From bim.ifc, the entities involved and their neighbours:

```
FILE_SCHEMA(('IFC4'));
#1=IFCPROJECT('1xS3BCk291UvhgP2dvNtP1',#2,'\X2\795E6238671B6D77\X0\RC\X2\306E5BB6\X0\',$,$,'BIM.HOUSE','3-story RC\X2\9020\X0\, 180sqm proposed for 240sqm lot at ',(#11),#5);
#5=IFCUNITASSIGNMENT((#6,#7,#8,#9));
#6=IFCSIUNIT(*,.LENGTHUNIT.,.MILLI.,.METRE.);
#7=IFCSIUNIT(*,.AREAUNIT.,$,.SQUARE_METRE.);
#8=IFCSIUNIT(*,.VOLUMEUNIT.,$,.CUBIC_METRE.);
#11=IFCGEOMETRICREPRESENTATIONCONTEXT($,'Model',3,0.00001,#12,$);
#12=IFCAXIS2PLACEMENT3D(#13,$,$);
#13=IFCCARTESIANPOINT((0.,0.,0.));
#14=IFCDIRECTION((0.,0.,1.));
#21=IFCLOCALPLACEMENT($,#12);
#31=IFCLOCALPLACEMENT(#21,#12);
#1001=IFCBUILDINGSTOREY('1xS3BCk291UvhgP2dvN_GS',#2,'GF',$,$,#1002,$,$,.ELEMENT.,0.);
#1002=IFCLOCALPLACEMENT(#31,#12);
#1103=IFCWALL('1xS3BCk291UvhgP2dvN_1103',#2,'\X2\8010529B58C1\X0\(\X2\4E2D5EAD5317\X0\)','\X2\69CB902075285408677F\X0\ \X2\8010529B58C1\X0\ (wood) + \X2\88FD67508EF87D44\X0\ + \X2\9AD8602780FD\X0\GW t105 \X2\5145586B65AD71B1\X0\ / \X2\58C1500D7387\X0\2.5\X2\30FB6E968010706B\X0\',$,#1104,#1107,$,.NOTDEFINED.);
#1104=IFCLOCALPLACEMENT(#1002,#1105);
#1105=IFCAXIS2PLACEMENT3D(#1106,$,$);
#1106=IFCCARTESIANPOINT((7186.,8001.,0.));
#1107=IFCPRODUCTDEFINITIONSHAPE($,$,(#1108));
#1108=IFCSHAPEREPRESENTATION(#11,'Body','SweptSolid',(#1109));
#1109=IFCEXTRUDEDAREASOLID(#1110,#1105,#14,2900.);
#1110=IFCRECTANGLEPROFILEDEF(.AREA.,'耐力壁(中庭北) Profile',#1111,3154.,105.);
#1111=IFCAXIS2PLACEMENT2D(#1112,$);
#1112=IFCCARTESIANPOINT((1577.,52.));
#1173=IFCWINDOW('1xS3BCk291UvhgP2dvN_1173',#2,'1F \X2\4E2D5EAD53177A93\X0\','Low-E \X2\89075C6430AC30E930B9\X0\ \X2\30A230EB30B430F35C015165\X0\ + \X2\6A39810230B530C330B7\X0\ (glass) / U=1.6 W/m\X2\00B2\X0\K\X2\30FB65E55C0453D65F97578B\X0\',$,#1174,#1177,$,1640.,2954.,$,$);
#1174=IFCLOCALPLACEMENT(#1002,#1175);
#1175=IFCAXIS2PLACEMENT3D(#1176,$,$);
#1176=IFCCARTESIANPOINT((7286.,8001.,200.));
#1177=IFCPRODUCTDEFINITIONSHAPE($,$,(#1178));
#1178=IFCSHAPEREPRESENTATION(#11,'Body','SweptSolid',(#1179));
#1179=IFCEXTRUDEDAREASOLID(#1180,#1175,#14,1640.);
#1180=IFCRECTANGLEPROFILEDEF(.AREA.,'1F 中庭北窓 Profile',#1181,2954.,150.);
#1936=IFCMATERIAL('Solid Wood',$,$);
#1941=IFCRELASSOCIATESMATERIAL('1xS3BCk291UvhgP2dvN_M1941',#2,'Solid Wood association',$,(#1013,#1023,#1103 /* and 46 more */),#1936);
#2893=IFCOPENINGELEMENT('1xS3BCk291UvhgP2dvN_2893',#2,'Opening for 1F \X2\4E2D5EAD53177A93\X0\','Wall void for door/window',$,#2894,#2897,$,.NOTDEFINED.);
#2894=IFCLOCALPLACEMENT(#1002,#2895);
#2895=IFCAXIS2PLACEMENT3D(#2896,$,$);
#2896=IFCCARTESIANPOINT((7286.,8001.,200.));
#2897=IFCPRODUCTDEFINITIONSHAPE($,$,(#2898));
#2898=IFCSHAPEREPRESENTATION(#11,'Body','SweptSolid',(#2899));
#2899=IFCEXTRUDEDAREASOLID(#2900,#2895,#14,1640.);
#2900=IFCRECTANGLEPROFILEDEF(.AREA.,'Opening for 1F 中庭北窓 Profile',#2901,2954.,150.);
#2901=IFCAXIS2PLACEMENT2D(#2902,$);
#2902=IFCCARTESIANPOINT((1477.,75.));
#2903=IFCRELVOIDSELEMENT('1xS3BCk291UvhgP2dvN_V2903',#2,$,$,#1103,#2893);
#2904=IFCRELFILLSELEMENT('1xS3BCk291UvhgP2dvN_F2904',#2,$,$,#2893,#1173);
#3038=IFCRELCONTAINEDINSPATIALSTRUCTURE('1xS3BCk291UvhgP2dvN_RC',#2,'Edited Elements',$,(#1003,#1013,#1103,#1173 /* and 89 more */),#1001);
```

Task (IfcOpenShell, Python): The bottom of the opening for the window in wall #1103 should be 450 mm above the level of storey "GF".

```python
import numpy as np
import ifcopenshell
import ifcopenshell.api.geometry
import ifcopenshell.geom
import ifcopenshell.util.element
import ifcopenshell.util.placement
import ifcopenshell.util.shape
import ifcopenshell.util.unit

model = ifcopenshell.open("bim.ifc")
unit_scale = ifcopenshell.util.unit.calculate_unit_scale(model)

window = model.by_guid("1xS3BCk291UvhgP2dvN_1173")
opening = window.FillsVoids[0].RelatingOpeningElement
storey = ifcopenshell.util.element.get_container(window, ifc_class="IfcBuildingStorey")
level = ifcopenshell.util.placement.get_local_placement(storey.ObjectPlacement)[2, 3]

# The opening's origin need not be at the sill, so measure its lowest point.
shape = ifcopenshell.geom.create_shape(ifcopenshell.geom.settings(), opening)
bottom = ifcopenshell.util.shape.get_shape_bottom_elevation(shape, shape.geometry) / unit_scale
dz = level + 0.45 / unit_scale - bottom

shift = np.array([0.0, 0.0, dz])
# The window is not placed relative to its opening, so move both.
for product in (opening, window):
    matrix = ifcopenshell.util.placement.get_local_placement(product.ObjectPlacement)
    matrix[:3, 3] += shift
    ifcopenshell.api.geometry.edit_object_placement(model, product=product, matrix=matrix, is_si=False)

print(f"moved by {dz * unit_scale:+.3f} m")

model.write("bim_rev.ifc")
```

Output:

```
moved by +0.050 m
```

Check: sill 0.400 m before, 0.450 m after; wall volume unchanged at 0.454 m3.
